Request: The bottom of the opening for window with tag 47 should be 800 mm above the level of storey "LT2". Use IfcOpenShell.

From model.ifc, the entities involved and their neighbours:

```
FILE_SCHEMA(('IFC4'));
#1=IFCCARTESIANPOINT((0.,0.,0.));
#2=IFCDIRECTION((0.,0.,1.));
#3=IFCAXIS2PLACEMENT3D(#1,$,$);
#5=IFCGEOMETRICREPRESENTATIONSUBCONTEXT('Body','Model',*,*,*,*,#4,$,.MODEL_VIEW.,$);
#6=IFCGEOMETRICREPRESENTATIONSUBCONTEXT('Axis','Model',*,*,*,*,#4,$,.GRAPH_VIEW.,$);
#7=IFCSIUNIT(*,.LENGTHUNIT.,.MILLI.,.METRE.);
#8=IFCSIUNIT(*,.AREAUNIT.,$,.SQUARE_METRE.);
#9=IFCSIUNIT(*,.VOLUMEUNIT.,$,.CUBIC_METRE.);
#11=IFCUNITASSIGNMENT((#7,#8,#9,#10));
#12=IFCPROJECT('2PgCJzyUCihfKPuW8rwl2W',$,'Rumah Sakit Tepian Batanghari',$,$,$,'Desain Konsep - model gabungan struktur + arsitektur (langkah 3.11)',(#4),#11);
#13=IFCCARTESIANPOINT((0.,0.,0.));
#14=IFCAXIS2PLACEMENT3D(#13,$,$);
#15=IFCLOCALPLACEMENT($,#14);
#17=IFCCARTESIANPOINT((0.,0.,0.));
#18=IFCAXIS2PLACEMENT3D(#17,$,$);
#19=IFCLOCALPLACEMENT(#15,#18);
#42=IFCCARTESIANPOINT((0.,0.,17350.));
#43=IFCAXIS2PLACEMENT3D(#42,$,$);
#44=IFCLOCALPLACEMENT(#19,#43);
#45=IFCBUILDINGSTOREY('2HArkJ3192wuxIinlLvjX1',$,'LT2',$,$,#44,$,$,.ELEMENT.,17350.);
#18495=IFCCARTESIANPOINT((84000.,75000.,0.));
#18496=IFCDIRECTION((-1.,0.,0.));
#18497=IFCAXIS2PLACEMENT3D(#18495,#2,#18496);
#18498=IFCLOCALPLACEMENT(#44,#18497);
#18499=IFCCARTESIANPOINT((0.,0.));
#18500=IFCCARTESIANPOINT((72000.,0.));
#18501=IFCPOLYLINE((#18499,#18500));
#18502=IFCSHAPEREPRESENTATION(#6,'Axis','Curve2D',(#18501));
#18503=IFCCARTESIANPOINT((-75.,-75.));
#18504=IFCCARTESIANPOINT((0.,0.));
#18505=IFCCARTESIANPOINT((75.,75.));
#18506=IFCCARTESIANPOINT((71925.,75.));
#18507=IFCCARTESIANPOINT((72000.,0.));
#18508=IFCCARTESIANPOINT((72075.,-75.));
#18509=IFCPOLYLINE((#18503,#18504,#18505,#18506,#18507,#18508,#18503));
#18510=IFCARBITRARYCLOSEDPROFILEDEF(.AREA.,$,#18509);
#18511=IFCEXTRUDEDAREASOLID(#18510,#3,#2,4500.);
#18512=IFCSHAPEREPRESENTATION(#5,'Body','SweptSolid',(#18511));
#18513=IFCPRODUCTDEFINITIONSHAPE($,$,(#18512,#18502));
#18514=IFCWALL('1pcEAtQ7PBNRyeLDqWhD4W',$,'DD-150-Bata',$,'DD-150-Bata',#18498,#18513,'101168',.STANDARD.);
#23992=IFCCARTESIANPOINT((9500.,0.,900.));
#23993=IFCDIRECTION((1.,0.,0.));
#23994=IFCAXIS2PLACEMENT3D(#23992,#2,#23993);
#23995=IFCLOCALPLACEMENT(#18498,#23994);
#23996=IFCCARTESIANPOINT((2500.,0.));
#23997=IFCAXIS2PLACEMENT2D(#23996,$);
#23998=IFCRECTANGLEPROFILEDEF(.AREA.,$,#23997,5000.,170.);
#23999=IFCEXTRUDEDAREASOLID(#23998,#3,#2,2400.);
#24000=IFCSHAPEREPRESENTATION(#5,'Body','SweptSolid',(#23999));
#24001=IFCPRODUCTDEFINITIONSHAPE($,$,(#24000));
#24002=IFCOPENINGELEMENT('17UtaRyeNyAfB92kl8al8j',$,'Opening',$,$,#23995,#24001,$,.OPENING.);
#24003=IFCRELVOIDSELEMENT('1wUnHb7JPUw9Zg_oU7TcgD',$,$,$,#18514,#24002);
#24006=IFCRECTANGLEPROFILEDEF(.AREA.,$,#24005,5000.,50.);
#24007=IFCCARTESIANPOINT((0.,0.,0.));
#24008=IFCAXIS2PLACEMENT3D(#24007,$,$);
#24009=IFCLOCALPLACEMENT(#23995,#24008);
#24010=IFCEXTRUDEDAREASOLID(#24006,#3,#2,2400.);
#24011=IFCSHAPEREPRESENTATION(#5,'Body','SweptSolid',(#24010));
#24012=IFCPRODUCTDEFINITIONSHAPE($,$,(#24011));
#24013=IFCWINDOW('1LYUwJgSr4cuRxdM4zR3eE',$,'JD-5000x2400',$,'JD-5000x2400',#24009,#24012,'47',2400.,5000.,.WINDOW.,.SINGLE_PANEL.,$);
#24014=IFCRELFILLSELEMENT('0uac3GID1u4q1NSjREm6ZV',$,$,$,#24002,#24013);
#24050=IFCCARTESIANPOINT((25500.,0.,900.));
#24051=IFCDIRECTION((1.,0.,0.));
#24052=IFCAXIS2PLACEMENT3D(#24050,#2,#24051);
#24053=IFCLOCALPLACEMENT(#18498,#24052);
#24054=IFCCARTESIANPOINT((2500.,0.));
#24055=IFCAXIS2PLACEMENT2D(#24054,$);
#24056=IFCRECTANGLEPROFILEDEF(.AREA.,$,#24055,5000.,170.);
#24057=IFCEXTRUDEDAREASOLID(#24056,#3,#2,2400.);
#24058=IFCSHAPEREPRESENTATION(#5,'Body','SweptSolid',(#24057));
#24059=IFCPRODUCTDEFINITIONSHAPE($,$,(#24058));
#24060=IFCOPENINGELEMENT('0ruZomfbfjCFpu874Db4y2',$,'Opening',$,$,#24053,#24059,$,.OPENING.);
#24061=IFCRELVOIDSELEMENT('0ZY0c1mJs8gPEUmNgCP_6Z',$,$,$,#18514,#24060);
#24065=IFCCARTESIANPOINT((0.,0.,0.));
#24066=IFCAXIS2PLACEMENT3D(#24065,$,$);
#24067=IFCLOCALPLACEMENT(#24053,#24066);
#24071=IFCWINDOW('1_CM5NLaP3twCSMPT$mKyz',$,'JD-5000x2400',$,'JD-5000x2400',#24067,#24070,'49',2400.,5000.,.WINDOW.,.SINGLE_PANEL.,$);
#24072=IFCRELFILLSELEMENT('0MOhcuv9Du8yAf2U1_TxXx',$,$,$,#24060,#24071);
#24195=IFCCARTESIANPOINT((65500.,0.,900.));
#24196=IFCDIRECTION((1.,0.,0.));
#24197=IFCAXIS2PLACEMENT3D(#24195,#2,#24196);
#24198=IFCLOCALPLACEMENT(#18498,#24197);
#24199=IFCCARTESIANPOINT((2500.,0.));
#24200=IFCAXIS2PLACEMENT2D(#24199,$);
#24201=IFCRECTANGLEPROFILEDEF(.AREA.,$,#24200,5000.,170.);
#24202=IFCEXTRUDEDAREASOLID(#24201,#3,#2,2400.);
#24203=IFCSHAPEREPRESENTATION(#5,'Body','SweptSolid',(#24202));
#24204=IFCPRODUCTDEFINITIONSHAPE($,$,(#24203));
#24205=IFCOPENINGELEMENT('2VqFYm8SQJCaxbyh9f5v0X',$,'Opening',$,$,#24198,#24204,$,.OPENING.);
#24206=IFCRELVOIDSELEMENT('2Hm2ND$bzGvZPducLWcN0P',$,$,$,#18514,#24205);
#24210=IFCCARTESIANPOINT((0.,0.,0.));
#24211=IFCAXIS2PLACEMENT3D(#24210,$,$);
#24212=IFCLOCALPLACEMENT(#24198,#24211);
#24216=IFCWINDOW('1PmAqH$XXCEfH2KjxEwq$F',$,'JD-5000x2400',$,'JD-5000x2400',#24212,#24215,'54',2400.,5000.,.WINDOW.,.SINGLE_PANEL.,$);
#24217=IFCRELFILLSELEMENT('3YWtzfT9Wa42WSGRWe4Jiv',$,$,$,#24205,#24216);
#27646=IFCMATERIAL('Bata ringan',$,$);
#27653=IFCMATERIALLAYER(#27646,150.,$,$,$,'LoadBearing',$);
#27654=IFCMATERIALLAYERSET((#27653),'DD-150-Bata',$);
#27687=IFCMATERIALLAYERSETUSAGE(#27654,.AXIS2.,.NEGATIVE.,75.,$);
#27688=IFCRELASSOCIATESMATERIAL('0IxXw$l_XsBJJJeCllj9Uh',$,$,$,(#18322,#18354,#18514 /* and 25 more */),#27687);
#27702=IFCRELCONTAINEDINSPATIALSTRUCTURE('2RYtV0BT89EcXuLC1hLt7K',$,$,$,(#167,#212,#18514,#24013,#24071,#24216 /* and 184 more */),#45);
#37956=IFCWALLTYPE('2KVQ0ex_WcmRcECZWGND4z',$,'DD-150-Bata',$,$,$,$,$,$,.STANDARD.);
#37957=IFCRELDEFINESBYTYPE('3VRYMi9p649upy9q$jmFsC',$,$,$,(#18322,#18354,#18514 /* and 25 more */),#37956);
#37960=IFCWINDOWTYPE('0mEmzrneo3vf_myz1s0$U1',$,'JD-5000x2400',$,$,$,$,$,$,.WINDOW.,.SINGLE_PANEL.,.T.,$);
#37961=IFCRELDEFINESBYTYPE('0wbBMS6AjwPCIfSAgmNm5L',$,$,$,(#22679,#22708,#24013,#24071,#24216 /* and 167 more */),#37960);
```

```python
import numpy as np
import ifcopenshell
import ifcopenshell.api.geometry
import ifcopenshell.geom
import ifcopenshell.util.element
import ifcopenshell.util.placement
import ifcopenshell.util.shape
import ifcopenshell.util.unit

model = ifcopenshell.open("model.ifc")
unit_scale = ifcopenshell.util.unit.calculate_unit_scale(model)

window = model.by_guid("1LYUwJgSr4cuRxdM4zR3eE")
opening = window.FillsVoids[0].RelatingOpeningElement
storey = ifcopenshell.util.element.get_container(window, ifc_class="IfcBuildingStorey")
level = ifcopenshell.util.placement.get_local_placement(storey.ObjectPlacement)[2, 3]

# The opening's origin need not be at the sill, so measure its lowest point.
shape = ifcopenshell.geom.create_shape(ifcopenshell.geom.settings(), opening)
bottom = ifcopenshell.util.shape.get_shape_bottom_elevation(shape, shape.geometry) / unit_scale
dz = level + 0.8 / unit_scale - bottom

shift = np.array([0.0, 0.0, dz])
# The window is placed relative to its opening, so it follows when the opening moves.
matrix = ifcopenshell.util.placement.get_local_placement(opening.ObjectPlacement)
matrix[:3, 3] += shift
ifcopenshell.api.geometry.edit_object_placement(
    model, product=opening, matrix=matrix, is_si=False, should_transform_children=True
)

print(f"moved by {dz * unit_scale:+.3f} m")

model.write("model_updated.ifc")
```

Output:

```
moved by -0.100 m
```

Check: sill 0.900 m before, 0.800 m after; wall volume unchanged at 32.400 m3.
